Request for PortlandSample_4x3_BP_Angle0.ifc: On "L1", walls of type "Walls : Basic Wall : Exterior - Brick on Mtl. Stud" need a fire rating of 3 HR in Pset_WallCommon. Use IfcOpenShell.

First a look at what the model holds.

```python
import ifcopenshell
import ifcopenshell.util.element

model = ifcopenshell.open("PortlandSample_4x3_BP_Angle0.ifc")
print(model.schema)
storey = next(s for s in model.by_type("IfcBuildingStorey") if s.Name == "L1")
walls = [e for e in ifcopenshell.util.element.get_decomposition(storey) if e.is_a("IfcWall")]
seen = {}
for e in walls:
    element_type = ifcopenshell.util.element.get_type(e)
    key = (element_type.Name if element_type != e and element_type else None, ifcopenshell.util.element.get_pset(e, "Pset_WallCommon", "FireRating"))
    seen[key] = seen.get(key, 0) + 1
for (name, value), count in sorted(seen.items(), key=str):
    print(count, "x", name, "|", value)
```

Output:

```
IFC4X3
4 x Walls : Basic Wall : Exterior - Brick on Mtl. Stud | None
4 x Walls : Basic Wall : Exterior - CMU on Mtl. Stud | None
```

```python
import ifcopenshell
import ifcopenshell.api.pset
import ifcopenshell.util.element

model = ifcopenshell.open("PortlandSample_4x3_BP_Angle0.ifc")

storey = next(s for s in model.by_type("IfcBuildingStorey") if s.Name == "L1")
walls = [e for e in ifcopenshell.util.element.get_decomposition(storey) if e.is_a("IfcWall")]

count = 0
for e in walls:
    element_type = ifcopenshell.util.element.get_type(e)
    if element_type in (None, e) or element_type.Name != "Walls : Basic Wall : Exterior - Brick on Mtl. Stud":
        continue
    # add_pset returns the element's existing set when there is one.
    pset = ifcopenshell.api.pset.add_pset(model, product=e, name="Pset_WallCommon")
    ifcopenshell.api.pset.edit_pset(model, pset=pset, properties={"FireRating": "3 HR"})
    count += 1

print(count, "walls updated")

model.write("PortlandSample_4x3_BP_Angle0_updated.ifc")
```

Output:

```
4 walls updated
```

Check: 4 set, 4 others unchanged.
